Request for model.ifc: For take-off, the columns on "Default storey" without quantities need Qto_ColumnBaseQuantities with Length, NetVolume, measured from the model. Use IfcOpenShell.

First a look at what the model holds.

```python
import ifcopenshell
import ifcopenshell.util.element
import ifcopenshell.util.unit

model = ifcopenshell.open("model.ifc")
print(model.schema)
for unit_type in ("LENGTHUNIT", "AREAUNIT", "VOLUMEUNIT"):
    print(unit_type, ifcopenshell.util.unit.calculate_unit_scale(model, unit_type))
storey = next(s for s in model.by_type("IfcBuildingStorey") if s.Name == "Default storey")
columns = [e for e in ifcopenshell.util.element.get_decomposition(storey) if e.is_a("IfcColumn")]
for e in sorted(columns, key=lambda e: e.id()):
    print(e.id(), e.is_a(), e.Name, list(ifcopenshell.util.element.get_psets(e, qtos_only=True)), sep=" | ")
```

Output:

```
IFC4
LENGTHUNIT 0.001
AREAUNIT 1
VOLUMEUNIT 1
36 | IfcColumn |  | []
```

```python
import ifcopenshell
import ifcopenshell.api.pset
import ifcopenshell.geom
import ifcopenshell.util.element
import ifcopenshell.util.shape
import ifcopenshell.util.unit

model = ifcopenshell.open("model.ifc")
unit_scale = ifcopenshell.util.unit.calculate_unit_scale(model)
volume_scale = ifcopenshell.util.unit.calculate_unit_scale(model, "VOLUMEUNIT")
settings = ifcopenshell.geom.settings()

storey = next(s for s in model.by_type("IfcBuildingStorey") if s.Name == "Default storey")
columns = [e for e in ifcopenshell.util.element.get_decomposition(storey) if e.is_a("IfcColumn")]

for e in sorted(columns, key=lambda e: e.id()):
    if ifcopenshell.util.element.get_psets(e, qtos_only=True, should_inherit=False):
        continue
    # Geometry comes back in metres, in the element's own axes.
    shape = ifcopenshell.geom.create_shape(settings, e)
    values = {
        "Length": ifcopenshell.util.shape.get_z(shape.geometry) / unit_scale,
        "NetVolume": ifcopenshell.util.shape.get_volume(shape.geometry) / volume_scale,
    }
    qto = ifcopenshell.api.pset.add_qto(model, product=e, name="Qto_ColumnBaseQuantities")
    ifcopenshell.api.pset.edit_qto(model, qto=qto, properties=values)
    print(e.id(), {k: round(v, 3) for k, v in values.items()})

model.write("model_edited.ifc")
```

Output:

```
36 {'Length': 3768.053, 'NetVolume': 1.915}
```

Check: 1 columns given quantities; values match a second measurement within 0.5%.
